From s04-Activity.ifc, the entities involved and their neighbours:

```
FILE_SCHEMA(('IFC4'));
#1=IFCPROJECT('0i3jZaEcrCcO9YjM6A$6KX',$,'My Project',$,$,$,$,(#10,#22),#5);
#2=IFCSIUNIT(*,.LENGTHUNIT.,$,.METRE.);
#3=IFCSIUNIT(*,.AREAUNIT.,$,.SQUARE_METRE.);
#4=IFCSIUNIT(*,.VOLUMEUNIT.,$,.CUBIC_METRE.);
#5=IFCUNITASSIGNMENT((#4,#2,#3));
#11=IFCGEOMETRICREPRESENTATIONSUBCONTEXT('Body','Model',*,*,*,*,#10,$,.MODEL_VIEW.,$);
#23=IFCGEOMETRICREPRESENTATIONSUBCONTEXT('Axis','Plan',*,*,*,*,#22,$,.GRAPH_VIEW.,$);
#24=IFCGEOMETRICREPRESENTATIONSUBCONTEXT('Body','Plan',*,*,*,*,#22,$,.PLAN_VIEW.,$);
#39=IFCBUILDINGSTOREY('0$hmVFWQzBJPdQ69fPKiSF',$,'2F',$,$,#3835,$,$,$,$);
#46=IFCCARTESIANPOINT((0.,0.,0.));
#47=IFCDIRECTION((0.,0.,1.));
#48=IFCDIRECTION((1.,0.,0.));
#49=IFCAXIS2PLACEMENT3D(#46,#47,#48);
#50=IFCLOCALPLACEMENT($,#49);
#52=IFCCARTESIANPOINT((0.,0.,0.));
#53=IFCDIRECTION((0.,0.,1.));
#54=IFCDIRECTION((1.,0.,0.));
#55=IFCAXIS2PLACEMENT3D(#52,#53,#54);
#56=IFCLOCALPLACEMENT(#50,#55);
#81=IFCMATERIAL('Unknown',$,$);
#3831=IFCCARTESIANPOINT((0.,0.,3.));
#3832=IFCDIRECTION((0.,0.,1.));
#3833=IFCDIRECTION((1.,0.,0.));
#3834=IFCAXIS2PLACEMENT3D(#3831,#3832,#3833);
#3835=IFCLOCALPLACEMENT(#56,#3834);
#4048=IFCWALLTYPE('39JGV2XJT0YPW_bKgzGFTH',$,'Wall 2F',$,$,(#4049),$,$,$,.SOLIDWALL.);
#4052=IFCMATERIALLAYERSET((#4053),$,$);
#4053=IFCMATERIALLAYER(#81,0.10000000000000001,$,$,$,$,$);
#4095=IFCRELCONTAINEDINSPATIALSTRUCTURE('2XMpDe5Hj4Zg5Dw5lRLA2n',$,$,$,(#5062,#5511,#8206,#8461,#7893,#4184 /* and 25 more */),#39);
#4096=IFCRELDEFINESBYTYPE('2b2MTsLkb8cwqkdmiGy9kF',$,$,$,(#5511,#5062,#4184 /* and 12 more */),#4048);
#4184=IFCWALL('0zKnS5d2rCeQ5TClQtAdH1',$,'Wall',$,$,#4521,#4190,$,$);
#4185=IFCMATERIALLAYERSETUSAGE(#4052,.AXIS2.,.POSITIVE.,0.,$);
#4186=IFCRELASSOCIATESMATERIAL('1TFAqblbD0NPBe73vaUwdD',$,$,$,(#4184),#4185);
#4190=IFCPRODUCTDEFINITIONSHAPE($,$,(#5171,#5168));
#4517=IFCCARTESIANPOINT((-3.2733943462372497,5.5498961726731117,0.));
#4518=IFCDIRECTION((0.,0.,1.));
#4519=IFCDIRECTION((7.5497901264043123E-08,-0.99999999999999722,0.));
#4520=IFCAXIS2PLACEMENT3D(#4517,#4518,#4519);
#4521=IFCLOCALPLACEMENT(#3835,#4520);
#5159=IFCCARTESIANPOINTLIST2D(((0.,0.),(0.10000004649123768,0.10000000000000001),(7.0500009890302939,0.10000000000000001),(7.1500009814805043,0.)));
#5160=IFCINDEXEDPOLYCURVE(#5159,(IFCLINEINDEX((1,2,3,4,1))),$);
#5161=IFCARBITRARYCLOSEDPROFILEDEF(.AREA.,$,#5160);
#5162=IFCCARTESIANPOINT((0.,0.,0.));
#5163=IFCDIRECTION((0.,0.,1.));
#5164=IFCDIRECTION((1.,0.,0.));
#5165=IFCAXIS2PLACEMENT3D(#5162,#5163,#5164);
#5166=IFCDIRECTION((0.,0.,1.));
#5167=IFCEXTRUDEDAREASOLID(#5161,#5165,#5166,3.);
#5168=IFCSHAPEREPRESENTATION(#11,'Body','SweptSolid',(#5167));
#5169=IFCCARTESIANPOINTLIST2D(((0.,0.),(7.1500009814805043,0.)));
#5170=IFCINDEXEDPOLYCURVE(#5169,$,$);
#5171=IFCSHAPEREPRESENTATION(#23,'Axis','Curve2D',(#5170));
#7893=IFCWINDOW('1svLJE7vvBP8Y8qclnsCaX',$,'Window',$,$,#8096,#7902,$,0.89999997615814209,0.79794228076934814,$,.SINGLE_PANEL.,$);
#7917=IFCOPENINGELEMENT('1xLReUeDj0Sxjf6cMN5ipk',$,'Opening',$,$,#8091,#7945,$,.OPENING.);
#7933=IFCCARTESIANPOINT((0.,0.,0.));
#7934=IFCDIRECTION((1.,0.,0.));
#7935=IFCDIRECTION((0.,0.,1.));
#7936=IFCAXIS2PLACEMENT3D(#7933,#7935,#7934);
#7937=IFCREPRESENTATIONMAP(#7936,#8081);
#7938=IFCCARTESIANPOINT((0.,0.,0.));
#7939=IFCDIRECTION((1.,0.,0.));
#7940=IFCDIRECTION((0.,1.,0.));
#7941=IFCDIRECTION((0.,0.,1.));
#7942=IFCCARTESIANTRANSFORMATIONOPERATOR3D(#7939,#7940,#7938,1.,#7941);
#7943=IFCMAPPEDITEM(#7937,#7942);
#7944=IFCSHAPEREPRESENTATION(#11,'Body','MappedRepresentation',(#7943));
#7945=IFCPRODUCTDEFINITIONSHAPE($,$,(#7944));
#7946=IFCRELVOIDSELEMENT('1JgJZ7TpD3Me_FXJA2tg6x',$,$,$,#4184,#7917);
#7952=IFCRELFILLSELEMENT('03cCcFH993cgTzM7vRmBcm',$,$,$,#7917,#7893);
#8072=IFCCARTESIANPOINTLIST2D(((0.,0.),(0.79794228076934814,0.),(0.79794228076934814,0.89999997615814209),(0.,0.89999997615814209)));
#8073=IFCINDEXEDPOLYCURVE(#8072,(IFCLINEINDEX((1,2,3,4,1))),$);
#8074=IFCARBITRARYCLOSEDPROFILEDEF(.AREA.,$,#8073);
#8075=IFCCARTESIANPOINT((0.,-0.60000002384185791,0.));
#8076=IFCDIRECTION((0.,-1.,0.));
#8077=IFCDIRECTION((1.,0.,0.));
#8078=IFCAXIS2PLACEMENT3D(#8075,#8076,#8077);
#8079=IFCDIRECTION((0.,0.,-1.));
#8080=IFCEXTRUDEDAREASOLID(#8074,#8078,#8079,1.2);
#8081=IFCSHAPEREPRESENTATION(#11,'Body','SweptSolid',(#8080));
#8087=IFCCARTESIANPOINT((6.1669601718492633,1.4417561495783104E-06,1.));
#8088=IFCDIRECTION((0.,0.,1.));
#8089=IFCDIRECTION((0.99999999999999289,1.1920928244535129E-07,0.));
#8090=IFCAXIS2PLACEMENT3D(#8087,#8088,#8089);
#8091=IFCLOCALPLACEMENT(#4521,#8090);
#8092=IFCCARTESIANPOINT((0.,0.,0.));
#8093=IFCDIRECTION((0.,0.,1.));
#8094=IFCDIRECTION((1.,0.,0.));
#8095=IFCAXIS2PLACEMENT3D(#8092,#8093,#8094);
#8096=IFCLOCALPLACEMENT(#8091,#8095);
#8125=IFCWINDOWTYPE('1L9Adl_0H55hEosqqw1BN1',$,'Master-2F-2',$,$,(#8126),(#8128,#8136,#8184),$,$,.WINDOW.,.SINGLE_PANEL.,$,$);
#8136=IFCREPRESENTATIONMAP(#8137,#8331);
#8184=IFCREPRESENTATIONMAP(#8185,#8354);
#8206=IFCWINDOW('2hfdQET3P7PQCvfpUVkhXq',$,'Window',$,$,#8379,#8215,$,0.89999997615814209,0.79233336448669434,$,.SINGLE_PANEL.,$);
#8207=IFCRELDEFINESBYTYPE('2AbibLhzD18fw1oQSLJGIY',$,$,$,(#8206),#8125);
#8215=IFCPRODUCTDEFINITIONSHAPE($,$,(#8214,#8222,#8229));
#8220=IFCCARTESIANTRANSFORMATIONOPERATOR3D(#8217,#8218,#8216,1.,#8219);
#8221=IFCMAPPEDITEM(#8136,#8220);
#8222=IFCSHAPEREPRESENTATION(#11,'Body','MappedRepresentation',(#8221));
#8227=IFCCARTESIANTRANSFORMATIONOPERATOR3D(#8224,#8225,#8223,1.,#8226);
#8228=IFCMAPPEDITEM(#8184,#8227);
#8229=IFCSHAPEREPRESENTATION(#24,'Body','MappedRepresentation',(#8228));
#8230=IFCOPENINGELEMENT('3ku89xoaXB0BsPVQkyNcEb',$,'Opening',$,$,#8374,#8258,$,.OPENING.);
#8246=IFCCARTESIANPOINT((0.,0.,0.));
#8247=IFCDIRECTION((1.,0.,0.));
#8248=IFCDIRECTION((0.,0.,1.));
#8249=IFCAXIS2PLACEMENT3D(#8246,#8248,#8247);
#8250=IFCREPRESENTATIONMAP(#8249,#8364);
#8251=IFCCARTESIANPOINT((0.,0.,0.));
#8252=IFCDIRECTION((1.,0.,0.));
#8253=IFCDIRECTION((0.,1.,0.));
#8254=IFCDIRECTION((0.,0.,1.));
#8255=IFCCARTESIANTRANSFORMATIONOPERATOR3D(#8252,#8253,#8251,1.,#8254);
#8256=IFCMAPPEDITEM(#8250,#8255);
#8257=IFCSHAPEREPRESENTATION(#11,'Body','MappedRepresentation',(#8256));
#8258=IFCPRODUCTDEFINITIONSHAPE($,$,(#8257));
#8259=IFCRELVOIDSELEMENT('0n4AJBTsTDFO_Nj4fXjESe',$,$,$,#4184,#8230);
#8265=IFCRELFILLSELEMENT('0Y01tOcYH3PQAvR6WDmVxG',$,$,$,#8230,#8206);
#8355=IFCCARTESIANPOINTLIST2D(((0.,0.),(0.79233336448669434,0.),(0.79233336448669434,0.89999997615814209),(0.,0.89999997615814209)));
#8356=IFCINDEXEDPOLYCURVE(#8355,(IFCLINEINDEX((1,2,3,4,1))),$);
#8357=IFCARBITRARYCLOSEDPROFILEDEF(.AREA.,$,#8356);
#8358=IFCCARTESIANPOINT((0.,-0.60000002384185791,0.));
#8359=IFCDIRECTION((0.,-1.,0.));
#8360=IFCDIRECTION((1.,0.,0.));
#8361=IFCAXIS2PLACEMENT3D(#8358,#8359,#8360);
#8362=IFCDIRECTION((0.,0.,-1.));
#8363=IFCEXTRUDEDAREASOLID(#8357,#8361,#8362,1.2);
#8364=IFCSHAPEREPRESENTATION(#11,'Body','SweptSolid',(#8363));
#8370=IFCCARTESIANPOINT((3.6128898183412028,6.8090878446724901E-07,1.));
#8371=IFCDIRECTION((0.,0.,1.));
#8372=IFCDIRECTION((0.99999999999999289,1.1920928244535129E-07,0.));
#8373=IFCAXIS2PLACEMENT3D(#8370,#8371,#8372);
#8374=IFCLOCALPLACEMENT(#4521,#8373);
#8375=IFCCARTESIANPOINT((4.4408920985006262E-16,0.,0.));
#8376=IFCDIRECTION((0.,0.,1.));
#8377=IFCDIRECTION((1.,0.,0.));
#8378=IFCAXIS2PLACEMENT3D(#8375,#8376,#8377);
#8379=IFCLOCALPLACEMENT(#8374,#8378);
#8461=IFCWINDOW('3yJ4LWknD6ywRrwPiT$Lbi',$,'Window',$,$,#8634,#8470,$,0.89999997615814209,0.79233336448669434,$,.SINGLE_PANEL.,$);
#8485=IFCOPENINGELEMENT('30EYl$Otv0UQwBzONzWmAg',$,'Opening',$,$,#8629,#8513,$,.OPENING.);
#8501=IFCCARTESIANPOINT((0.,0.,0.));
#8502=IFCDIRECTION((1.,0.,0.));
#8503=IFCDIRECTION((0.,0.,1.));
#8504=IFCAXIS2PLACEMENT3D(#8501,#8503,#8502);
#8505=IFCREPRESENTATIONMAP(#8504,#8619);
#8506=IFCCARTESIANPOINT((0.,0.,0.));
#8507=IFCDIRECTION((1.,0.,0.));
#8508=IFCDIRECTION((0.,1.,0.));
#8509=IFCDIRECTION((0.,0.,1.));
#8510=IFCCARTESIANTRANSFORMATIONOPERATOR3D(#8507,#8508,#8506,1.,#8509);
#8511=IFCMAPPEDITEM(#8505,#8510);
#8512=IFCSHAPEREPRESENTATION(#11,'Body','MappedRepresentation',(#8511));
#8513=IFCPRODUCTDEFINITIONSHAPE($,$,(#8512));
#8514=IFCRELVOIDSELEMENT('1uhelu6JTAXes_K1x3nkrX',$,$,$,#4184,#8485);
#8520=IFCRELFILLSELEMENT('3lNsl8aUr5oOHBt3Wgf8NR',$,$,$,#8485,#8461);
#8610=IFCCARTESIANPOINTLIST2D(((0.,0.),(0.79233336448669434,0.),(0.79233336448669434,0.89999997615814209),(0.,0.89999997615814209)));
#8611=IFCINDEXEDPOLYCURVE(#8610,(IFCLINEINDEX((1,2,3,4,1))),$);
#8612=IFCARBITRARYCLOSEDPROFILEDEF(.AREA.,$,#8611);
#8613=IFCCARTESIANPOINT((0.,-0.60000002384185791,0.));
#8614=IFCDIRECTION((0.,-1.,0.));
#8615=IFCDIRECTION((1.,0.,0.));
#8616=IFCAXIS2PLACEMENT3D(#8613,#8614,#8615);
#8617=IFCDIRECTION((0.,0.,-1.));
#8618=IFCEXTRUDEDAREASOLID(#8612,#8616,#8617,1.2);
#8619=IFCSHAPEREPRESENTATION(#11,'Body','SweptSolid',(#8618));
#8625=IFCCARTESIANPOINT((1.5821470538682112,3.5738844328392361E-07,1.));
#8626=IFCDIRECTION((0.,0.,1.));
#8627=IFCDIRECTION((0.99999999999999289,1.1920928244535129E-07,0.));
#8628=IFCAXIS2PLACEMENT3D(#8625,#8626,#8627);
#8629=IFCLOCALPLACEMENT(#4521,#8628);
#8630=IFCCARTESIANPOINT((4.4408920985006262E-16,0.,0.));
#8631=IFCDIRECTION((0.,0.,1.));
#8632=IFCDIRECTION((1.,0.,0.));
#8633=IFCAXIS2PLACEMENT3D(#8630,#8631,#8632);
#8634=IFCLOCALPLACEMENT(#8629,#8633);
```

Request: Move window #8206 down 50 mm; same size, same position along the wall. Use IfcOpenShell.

```python
import numpy as np
import ifcopenshell
import ifcopenshell.api.geometry
import ifcopenshell.util.placement
import ifcopenshell.util.unit

model = ifcopenshell.open("s04-Activity.ifc")
unit_scale = ifcopenshell.util.unit.calculate_unit_scale(model)

window = model.by_guid("2hfdQET3P7PQCvfpUVkhXq")
opening = window.FillsVoids[0].RelatingOpeningElement
dz = -0.05

shift = np.array([0.0, 0.0, dz])
# The window is placed relative to its opening, so it follows when the opening moves.
matrix = ifcopenshell.util.placement.get_local_placement(opening.ObjectPlacement)
matrix[:3, 3] += shift
ifcopenshell.api.geometry.edit_object_placement(
    model, product=opening, matrix=matrix, is_si=False, should_transform_children=True
)

print(f"moved by {dz * unit_scale:+.3f} m")

model.write("s04-Activity_rev.ifc")
```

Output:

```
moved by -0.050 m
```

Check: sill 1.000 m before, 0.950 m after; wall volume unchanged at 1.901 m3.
